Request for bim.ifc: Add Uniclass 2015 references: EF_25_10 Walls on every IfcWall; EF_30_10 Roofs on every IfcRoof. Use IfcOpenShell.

First a look at what the model holds.

```python
import ifcopenshell

model = ifcopenshell.open("bim.ifc")
print(model.schema)
print("classifications:", [c.Name for c in model.by_type("IfcClassification")])
for ifc_class in ("IfcDoor", "IfcRoof", "IfcStair", "IfcWall", "IfcWindow"):
    print(ifc_class, len(model.by_type(ifc_class)))
```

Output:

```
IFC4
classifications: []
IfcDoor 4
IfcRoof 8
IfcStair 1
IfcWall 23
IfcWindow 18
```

```python
import ifcopenshell
import ifcopenshell.api.classification

model = ifcopenshell.open("bim.ifc")

system = ifcopenshell.api.classification.add_classification(model, classification="Uniclass 2015")

codes = {
    "IfcWall": ("EF_25_10", "Walls"),
    "IfcRoof": ("EF_30_10", "Roofs"),
}
for ifc_class, (code, name) in codes.items():
    products = model.by_type(ifc_class)
    ifcopenshell.api.classification.add_reference(
        model, products=products, classification=system, identification=code, name=name
    )
    print(code, len(products))

model.write("bim_edited.ifc")
```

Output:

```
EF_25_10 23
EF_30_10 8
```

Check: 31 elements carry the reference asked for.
